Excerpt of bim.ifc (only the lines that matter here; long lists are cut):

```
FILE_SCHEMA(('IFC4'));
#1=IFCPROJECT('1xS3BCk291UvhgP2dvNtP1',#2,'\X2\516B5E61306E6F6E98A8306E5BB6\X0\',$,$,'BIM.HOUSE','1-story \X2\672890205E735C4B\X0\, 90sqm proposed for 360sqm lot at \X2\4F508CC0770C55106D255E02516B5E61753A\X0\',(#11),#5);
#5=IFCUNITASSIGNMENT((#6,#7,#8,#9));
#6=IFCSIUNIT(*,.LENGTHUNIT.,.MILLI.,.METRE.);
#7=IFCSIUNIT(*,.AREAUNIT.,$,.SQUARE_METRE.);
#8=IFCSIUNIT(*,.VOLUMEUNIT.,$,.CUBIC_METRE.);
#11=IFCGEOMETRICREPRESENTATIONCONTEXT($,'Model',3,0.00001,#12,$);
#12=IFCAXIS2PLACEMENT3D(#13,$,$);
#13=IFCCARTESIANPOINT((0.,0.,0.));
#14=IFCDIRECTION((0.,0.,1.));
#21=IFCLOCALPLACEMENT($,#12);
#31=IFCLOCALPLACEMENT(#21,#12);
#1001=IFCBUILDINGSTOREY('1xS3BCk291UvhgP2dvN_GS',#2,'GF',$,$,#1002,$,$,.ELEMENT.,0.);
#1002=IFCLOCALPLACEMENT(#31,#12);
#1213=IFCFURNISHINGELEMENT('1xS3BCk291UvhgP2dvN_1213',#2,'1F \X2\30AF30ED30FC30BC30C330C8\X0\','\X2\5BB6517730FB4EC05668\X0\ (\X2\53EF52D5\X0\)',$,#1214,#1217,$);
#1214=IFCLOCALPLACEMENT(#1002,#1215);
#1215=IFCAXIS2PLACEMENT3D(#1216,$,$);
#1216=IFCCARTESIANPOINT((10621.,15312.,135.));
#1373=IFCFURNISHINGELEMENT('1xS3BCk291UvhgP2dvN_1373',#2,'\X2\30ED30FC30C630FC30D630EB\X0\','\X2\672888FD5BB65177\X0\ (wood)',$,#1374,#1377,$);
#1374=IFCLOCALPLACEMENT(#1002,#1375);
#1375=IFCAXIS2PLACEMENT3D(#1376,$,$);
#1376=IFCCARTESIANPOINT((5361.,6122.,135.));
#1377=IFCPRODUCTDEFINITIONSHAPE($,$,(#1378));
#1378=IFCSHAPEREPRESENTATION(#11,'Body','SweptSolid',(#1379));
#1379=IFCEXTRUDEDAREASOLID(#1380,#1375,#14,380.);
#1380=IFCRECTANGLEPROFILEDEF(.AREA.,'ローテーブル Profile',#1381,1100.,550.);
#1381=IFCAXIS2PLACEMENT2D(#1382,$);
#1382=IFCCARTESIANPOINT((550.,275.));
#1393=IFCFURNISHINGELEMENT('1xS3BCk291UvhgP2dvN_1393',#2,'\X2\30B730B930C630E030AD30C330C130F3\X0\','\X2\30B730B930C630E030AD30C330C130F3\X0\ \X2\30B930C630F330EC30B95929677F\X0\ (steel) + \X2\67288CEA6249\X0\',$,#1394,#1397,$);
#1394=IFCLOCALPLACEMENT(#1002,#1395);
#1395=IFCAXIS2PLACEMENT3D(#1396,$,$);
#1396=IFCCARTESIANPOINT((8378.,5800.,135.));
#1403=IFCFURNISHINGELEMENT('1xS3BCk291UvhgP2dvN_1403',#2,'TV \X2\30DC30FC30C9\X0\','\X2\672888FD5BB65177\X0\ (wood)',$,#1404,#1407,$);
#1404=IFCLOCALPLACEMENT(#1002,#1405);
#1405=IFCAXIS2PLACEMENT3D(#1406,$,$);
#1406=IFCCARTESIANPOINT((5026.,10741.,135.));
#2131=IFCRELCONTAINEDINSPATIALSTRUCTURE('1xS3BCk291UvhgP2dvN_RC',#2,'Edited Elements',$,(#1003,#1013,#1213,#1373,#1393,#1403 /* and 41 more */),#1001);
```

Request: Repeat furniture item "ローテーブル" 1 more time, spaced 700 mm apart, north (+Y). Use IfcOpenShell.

```python
import numpy as np
import ifcopenshell
import ifcopenshell.api.geometry
import ifcopenshell.api.root
import ifcopenshell.util.element
import ifcopenshell.util.placement

model = ifcopenshell.open("bim.ifc")


def reuse_history(source, copy):
    """copy_class also copies each property set's owner history, people and application; keep the originals."""
    for rel in copy.IsDefinedBy:
        if rel.is_a("IfcRelDefinesByProperties") and (history := rel.RelatingPropertyDefinition.OwnerHistory):
            rel.RelatingPropertyDefinition.OwnerHistory = source.OwnerHistory
            ifcopenshell.util.element.remove_deep2(model, history)


source = model.by_id(1373)
base = ifcopenshell.util.placement.get_local_placement(source.ObjectPlacement)
step = np.array([0.0, 1.0, 0.0]) * 700.0

for i in range(1, 2):
    copy = ifcopenshell.api.root.copy_class(model, product=source)
    copy.Representation = ifcopenshell.util.element.copy_deep(
        model, source.Representation, exclude=["IfcGeometricRepresentationContext", "IfcRepresentationMap"]
    )
    reuse_history(source, copy)
    matrix = base.copy()
    matrix[:3, 3] += i * step
    print("added at", matrix[:3, 3].round(3) + 0.0)
    ifcopenshell.api.geometry.edit_object_placement(model, product=copy, matrix=matrix, is_si=False)

model.write("bim_v2.ifc")
```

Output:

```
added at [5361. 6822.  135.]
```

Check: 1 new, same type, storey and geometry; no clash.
